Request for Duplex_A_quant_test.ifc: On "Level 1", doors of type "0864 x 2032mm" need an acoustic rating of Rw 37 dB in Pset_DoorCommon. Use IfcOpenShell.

First a look at what the model holds.

```python
import ifcopenshell
import ifcopenshell.util.element

model = ifcopenshell.open("Duplex_A_quant_test.ifc")
print(model.schema)
storey = next(s for s in model.by_type("IfcBuildingStorey") if s.Name == "Level 1")
doors = [e for e in ifcopenshell.util.element.get_decomposition(storey) if e.is_a("IfcDoor")]
seen = {}
for e in doors:
    element_type = ifcopenshell.util.element.get_type(e)
    key = (element_type.Name if element_type != e and element_type else None, ifcopenshell.util.element.get_pset(e, "Pset_DoorCommon", "AcousticRating"))
    seen[key] = seen.get(key, 0) + 1
for (name, value), count in sorted(seen.items(), key=str):
    print(count, "x", name, "|", value)
```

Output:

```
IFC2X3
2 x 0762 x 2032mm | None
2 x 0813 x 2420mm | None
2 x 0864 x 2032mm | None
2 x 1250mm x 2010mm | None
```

```python
import ifcopenshell
import ifcopenshell.api.pset
import ifcopenshell.util.element

model = ifcopenshell.open("Duplex_A_quant_test.ifc")

storey = next(s for s in model.by_type("IfcBuildingStorey") if s.Name == "Level 1")
doors = [e for e in ifcopenshell.util.element.get_decomposition(storey) if e.is_a("IfcDoor")]

count = 0
for e in doors:
    element_type = ifcopenshell.util.element.get_type(e)
    if element_type in (None, e) or element_type.Name != "0864 x 2032mm":
        continue
    # add_pset returns the element's existing set when there is one.
    pset = ifcopenshell.api.pset.add_pset(model, product=e, name="Pset_DoorCommon")
    ifcopenshell.api.pset.edit_pset(model, pset=pset, properties={"AcousticRating": "Rw 37 dB"})
    count += 1

print(count, "doors updated")

model.write("Duplex_A_quant_test_edited.ifc")
```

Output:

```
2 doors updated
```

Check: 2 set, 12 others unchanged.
